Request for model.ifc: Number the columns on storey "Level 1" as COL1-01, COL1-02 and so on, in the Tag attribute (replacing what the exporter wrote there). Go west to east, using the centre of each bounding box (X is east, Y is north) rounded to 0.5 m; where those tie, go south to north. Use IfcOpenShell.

First a look at what the model holds.

```python
import ifcopenshell
import ifcopenshell.util.element
import ifcopenshell.util.placement

model = ifcopenshell.open("model.ifc")
print(model.schema)
storey = next(s for s in model.by_type("IfcBuildingStorey") if s.Name == "Level 1")
columns = [e for e in ifcopenshell.util.element.get_decomposition(storey) if e.is_a("IfcColumn")]
for e in sorted(columns, key=lambda e: e.id()):
    origin = ifcopenshell.util.placement.get_local_placement(e.ObjectPlacement)[:3, 3]
    print(e.id(), e.Tag, e.Name, origin.round(2) + 0.0, sep=" | ")
```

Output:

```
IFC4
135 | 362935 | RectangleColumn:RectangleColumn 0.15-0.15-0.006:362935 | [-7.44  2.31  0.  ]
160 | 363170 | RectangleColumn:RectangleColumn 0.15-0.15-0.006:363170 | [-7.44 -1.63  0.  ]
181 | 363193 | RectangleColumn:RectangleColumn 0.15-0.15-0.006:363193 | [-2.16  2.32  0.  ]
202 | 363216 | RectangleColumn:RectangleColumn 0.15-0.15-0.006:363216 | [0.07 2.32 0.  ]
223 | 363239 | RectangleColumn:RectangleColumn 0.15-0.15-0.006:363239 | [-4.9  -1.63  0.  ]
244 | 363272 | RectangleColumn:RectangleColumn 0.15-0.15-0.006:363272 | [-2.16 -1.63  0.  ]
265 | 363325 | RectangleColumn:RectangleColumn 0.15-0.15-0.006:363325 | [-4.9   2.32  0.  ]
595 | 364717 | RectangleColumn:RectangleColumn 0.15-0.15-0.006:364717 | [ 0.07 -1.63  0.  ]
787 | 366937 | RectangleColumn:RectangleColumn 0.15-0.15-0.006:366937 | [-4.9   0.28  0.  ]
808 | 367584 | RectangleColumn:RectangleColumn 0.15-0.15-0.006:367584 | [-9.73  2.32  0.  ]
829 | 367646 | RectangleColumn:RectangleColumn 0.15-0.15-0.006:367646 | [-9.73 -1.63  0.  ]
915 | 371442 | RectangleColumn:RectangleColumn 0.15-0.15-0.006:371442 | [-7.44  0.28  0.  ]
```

```python
import ifcopenshell
import ifcopenshell.geom
import ifcopenshell.util.element
import ifcopenshell.util.shape

model = ifcopenshell.open("model.ifc")
settings = ifcopenshell.geom.settings()
settings.set("use-world-coords", True)


def centre(element):
    shape = ifcopenshell.geom.create_shape(settings, element)
    return ifcopenshell.util.shape.get_bbox_centroid(shape.geometry)


storey = next(s for s in model.by_type("IfcBuildingStorey") if s.Name == "Level 1")
columns = [e for e in ifcopenshell.util.element.get_decomposition(storey) if e.is_a("IfcColumn")]

# Insertion points can sit at a corner or the storey origin, so sort by the geometry (in metres).
centres = {e: centre(e) for e in columns}
columns.sort(key=lambda e: (round(centres[e][0] / 0.5), centres[e][1]))

for i, e in enumerate(columns, start=1):
    number = f"COL1-{i:02d}"
    e.Tag = number
    print(e.id(), number)

model.write("model_updated.ifc")
```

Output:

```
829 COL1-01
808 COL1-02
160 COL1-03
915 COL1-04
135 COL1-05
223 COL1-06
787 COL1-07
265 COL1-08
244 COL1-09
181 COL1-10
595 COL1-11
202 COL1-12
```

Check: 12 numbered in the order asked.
